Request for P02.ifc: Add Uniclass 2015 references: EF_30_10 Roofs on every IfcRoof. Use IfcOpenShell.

First a look at what the model holds.

```python
import ifcopenshell

model = ifcopenshell.open("P02.ifc")
print(model.schema)
print("classifications:", [c.Name for c in model.by_type("IfcClassification")])
for ifc_class in ("IfcDoor", "IfcRoof", "IfcStair", "IfcWall", "IfcWindow"):
    print(ifc_class, len(model.by_type(ifc_class)))
```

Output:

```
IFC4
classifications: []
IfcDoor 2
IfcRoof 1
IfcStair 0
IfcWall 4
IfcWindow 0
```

```python
import ifcopenshell
import ifcopenshell.api.classification

model = ifcopenshell.open("P02.ifc")

system = ifcopenshell.api.classification.add_classification(model, classification="Uniclass 2015")

codes = {
    "IfcRoof": ("EF_30_10", "Roofs"),
}
for ifc_class, (code, name) in codes.items():
    products = model.by_type(ifc_class)
    ifcopenshell.api.classification.add_reference(
        model, products=products, classification=system, identification=code, name=name
    )
    print(code, len(products))

model.write("P02_rev.ifc")
```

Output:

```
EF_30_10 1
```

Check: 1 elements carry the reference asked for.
